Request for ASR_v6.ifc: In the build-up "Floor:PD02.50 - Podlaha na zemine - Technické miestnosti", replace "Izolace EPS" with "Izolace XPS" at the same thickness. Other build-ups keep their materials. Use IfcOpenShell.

First a look at what the model holds.

```python
import ifcopenshell
import ifcopenshell.util.element

model = ifcopenshell.open("ASR_v6.ifc")
print(model.schema)
for layer_set in model.by_type("IfcMaterialLayerSet"):
    if layer_set.LayerSetName == "Floor:PD02.50 - Podlaha na zemine - Technické miestnosti":
        for layer in layer_set.MaterialLayers:
            print(layer.id(), layer.Material and layer.Material.Name, layer.LayerThickness, sep=" | ")
        print(len(ifcopenshell.util.element.get_elements_by_material(model, layer_set)), "elements and types use it")
print(sorted(m.Name for m in model.by_type("IfcMaterial") if m.Name)[:60])
```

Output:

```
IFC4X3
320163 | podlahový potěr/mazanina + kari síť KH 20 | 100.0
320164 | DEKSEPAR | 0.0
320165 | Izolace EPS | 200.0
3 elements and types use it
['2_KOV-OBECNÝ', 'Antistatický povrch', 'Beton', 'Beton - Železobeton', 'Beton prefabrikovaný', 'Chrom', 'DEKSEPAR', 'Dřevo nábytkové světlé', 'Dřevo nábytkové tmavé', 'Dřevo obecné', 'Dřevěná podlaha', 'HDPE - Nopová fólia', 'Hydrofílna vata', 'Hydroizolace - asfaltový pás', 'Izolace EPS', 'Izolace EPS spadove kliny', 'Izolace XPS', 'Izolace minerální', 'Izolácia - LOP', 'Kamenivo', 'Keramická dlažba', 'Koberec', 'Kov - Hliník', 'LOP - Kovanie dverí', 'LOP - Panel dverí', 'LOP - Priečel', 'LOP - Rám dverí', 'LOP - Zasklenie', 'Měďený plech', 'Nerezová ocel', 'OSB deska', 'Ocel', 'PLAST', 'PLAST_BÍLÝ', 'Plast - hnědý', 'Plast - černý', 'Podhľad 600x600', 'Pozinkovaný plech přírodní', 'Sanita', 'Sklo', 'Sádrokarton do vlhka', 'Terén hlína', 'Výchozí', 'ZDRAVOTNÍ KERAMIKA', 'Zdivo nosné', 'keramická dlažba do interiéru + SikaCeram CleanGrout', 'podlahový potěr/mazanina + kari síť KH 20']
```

```python
import ifcopenshell
import ifcopenshell.api.material

model = ifcopenshell.open("ASR_v6.ifc")

layer_set = next(s for s in model.by_type("IfcMaterialLayerSet") if s.LayerSetName == "Floor:PD02.50 - Podlaha na zemine - Technické miestnosti")
layer = next(l for l in layer_set.MaterialLayers if l.Material and l.Material.Name == "Izolace EPS")
material = next(m for m in model.by_type("IfcMaterial") if m.Name == "Izolace XPS")

# Point this one layer at the other material; renaming the old one would change it everywhere.
ifcopenshell.api.material.edit_layer(model, layer=layer, attributes={"Name": material.Name}, material=material)

print([l.Material.Name if l.Material else None for l in layer_set.MaterialLayers])

model.write("ASR_v6_edited.ifc")
```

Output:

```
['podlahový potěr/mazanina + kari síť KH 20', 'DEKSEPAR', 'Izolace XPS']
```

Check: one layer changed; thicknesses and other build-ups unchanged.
